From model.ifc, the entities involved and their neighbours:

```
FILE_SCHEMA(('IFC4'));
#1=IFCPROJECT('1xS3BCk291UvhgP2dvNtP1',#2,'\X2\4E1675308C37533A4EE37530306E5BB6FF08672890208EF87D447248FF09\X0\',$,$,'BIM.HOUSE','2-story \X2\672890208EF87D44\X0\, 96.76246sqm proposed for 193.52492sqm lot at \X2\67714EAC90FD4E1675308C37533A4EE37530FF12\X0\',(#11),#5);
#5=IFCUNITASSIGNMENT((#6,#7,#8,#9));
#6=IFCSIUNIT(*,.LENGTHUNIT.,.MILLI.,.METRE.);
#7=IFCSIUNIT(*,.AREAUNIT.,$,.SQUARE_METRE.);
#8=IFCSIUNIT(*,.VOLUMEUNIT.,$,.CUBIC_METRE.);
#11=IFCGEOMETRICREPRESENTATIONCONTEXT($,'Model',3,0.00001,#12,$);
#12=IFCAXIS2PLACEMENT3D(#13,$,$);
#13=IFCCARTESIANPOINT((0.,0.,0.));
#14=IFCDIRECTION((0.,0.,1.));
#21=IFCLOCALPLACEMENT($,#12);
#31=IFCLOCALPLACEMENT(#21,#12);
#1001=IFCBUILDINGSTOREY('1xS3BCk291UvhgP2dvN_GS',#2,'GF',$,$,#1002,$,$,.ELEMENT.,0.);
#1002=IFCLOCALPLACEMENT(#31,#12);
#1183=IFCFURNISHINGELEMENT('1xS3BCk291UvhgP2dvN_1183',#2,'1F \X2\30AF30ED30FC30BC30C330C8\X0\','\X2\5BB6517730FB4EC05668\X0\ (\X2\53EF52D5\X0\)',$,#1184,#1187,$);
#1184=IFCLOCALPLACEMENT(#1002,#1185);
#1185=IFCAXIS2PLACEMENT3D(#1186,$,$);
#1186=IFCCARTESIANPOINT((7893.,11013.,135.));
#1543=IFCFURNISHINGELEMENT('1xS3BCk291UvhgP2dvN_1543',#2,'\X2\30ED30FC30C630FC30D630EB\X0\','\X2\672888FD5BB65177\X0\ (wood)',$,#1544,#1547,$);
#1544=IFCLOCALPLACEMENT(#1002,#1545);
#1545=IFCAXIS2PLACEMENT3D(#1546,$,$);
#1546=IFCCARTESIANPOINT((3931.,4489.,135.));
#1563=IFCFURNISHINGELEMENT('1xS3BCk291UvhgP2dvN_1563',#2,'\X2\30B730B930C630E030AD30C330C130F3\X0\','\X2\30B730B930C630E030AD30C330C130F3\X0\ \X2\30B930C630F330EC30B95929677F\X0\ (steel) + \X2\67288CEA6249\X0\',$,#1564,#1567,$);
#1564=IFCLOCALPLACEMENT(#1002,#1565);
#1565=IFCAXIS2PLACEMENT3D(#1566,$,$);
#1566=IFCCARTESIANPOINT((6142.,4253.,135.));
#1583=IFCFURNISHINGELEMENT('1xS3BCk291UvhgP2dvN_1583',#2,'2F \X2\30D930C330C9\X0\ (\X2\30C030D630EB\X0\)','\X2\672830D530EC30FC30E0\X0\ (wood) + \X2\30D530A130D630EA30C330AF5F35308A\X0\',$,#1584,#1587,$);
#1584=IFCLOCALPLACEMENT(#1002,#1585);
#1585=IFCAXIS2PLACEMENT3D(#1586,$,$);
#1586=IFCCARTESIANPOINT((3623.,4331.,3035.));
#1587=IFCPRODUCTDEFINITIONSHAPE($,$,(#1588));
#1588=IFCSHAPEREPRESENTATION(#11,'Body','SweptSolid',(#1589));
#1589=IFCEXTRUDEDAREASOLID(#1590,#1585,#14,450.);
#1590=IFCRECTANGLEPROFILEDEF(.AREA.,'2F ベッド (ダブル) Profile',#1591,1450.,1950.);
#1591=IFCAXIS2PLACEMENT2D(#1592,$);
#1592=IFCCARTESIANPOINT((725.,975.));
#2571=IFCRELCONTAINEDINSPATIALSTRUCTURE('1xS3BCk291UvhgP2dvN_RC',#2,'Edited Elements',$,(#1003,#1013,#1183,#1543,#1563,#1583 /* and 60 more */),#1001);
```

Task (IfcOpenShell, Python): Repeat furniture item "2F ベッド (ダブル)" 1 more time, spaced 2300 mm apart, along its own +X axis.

```python
import ifcopenshell
import ifcopenshell.api.geometry
import ifcopenshell.api.root
import ifcopenshell.util.element
import ifcopenshell.util.placement

model = ifcopenshell.open("model.ifc")


def reuse_history(source, copy):
    """copy_class also copies each property set's owner history, people and application; keep the originals."""
    for rel in copy.IsDefinedBy:
        if rel.is_a("IfcRelDefinesByProperties") and (history := rel.RelatingPropertyDefinition.OwnerHistory):
            rel.RelatingPropertyDefinition.OwnerHistory = source.OwnerHistory
            ifcopenshell.util.element.remove_deep2(model, history)


source = model.by_guid("1xS3BCk291UvhgP2dvN_1583")
base = ifcopenshell.util.placement.get_local_placement(source.ObjectPlacement)
step = base[:3, 0] * 2300.0

for i in range(1, 2):
    copy = ifcopenshell.api.root.copy_class(model, product=source)
    copy.Representation = ifcopenshell.util.element.copy_deep(
        model, source.Representation, exclude=["IfcGeometricRepresentationContext", "IfcRepresentationMap"]
    )
    reuse_history(source, copy)
    matrix = base.copy()
    matrix[:3, 3] += i * step
    print("added at", matrix[:3, 3].round(3) + 0.0)
    ifcopenshell.api.geometry.edit_object_placement(model, product=copy, matrix=matrix, is_si=False)

model.write("model_rev.ifc")
```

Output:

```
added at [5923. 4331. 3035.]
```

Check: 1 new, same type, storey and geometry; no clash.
